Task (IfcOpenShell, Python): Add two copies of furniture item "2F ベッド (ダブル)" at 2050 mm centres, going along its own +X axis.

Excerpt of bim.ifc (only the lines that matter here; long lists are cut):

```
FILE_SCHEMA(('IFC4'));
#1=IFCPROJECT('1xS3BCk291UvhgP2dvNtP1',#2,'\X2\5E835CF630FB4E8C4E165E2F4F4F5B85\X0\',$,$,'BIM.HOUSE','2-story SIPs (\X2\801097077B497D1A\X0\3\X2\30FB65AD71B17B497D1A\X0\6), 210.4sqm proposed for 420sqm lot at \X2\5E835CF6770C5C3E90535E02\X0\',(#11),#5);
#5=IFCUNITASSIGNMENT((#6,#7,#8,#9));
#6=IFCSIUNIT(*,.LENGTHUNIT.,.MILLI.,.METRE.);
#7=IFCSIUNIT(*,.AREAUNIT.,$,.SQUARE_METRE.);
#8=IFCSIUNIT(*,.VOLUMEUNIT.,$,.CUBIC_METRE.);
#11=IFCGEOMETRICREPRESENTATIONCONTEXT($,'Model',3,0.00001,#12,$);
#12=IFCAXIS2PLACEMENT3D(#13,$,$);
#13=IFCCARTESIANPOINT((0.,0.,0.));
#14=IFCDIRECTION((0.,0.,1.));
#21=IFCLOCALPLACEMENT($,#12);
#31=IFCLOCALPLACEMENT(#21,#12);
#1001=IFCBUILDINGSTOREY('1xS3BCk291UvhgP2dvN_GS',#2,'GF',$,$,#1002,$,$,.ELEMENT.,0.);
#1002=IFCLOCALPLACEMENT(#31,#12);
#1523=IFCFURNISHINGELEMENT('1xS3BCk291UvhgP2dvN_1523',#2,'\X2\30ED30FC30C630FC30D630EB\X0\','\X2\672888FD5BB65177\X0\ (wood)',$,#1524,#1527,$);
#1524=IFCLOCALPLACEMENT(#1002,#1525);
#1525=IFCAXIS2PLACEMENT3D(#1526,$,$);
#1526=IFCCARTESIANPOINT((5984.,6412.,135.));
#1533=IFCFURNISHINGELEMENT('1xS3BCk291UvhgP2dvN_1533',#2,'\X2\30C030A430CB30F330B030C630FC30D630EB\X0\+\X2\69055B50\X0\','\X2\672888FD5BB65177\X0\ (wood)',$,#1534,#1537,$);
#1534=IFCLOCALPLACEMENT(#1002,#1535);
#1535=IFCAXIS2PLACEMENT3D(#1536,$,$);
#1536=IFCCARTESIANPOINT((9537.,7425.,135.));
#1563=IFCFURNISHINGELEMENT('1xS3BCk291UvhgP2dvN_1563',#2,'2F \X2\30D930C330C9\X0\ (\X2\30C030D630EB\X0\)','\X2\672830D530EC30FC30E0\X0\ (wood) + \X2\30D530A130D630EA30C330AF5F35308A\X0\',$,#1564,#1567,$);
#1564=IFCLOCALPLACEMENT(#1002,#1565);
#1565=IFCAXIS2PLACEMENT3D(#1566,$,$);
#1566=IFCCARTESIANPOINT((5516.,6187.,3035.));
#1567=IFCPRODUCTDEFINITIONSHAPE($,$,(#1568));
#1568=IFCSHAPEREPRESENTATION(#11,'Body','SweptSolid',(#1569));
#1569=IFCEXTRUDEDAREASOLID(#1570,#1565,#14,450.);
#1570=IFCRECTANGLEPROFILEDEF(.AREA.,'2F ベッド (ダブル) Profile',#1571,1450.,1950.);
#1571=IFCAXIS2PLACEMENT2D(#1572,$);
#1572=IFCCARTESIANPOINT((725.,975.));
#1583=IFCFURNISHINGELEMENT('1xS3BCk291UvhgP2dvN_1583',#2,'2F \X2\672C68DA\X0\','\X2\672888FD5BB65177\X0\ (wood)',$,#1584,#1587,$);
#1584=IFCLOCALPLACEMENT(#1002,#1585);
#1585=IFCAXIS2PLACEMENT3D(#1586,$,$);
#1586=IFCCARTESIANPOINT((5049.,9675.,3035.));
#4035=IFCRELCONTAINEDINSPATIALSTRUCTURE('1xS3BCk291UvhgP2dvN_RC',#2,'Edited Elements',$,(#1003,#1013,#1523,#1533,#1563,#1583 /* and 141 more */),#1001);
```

```python
import ifcopenshell
import ifcopenshell.api.geometry
import ifcopenshell.api.root
import ifcopenshell.util.element
import ifcopenshell.util.placement
import ifcopenshell.util.unit

model = ifcopenshell.open("bim.ifc")
unit_scale = ifcopenshell.util.unit.calculate_unit_scale(model)


def reuse_history(source, copy):
    """copy_class also copies each property set's owner history, people and application; keep the originals."""
    for rel in copy.IsDefinedBy:
        if rel.is_a("IfcRelDefinesByProperties") and (history := rel.RelatingPropertyDefinition.OwnerHistory):
            rel.RelatingPropertyDefinition.OwnerHistory = source.OwnerHistory
            ifcopenshell.util.element.remove_deep2(model, history)


source = model.by_guid("1xS3BCk291UvhgP2dvN_1563")
base = ifcopenshell.util.placement.get_local_placement(source.ObjectPlacement)
step = base[:3, 0] * 2.05 / unit_scale

for i in range(1, 3):
    copy = ifcopenshell.api.root.copy_class(model, product=source)
    copy.Representation = ifcopenshell.util.element.copy_deep(
        model, source.Representation, exclude=["IfcGeometricRepresentationContext", "IfcRepresentationMap"]
    )
    reuse_history(source, copy)
    matrix = base.copy()
    matrix[:3, 3] += i * step
    print("added at", matrix[:3, 3].round(3) + 0.0)
    ifcopenshell.api.geometry.edit_object_placement(model, product=copy, matrix=matrix, is_si=False)

model.write("bim_updated.ifc")
```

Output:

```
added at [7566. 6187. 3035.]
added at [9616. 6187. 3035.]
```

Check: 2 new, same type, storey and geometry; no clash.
